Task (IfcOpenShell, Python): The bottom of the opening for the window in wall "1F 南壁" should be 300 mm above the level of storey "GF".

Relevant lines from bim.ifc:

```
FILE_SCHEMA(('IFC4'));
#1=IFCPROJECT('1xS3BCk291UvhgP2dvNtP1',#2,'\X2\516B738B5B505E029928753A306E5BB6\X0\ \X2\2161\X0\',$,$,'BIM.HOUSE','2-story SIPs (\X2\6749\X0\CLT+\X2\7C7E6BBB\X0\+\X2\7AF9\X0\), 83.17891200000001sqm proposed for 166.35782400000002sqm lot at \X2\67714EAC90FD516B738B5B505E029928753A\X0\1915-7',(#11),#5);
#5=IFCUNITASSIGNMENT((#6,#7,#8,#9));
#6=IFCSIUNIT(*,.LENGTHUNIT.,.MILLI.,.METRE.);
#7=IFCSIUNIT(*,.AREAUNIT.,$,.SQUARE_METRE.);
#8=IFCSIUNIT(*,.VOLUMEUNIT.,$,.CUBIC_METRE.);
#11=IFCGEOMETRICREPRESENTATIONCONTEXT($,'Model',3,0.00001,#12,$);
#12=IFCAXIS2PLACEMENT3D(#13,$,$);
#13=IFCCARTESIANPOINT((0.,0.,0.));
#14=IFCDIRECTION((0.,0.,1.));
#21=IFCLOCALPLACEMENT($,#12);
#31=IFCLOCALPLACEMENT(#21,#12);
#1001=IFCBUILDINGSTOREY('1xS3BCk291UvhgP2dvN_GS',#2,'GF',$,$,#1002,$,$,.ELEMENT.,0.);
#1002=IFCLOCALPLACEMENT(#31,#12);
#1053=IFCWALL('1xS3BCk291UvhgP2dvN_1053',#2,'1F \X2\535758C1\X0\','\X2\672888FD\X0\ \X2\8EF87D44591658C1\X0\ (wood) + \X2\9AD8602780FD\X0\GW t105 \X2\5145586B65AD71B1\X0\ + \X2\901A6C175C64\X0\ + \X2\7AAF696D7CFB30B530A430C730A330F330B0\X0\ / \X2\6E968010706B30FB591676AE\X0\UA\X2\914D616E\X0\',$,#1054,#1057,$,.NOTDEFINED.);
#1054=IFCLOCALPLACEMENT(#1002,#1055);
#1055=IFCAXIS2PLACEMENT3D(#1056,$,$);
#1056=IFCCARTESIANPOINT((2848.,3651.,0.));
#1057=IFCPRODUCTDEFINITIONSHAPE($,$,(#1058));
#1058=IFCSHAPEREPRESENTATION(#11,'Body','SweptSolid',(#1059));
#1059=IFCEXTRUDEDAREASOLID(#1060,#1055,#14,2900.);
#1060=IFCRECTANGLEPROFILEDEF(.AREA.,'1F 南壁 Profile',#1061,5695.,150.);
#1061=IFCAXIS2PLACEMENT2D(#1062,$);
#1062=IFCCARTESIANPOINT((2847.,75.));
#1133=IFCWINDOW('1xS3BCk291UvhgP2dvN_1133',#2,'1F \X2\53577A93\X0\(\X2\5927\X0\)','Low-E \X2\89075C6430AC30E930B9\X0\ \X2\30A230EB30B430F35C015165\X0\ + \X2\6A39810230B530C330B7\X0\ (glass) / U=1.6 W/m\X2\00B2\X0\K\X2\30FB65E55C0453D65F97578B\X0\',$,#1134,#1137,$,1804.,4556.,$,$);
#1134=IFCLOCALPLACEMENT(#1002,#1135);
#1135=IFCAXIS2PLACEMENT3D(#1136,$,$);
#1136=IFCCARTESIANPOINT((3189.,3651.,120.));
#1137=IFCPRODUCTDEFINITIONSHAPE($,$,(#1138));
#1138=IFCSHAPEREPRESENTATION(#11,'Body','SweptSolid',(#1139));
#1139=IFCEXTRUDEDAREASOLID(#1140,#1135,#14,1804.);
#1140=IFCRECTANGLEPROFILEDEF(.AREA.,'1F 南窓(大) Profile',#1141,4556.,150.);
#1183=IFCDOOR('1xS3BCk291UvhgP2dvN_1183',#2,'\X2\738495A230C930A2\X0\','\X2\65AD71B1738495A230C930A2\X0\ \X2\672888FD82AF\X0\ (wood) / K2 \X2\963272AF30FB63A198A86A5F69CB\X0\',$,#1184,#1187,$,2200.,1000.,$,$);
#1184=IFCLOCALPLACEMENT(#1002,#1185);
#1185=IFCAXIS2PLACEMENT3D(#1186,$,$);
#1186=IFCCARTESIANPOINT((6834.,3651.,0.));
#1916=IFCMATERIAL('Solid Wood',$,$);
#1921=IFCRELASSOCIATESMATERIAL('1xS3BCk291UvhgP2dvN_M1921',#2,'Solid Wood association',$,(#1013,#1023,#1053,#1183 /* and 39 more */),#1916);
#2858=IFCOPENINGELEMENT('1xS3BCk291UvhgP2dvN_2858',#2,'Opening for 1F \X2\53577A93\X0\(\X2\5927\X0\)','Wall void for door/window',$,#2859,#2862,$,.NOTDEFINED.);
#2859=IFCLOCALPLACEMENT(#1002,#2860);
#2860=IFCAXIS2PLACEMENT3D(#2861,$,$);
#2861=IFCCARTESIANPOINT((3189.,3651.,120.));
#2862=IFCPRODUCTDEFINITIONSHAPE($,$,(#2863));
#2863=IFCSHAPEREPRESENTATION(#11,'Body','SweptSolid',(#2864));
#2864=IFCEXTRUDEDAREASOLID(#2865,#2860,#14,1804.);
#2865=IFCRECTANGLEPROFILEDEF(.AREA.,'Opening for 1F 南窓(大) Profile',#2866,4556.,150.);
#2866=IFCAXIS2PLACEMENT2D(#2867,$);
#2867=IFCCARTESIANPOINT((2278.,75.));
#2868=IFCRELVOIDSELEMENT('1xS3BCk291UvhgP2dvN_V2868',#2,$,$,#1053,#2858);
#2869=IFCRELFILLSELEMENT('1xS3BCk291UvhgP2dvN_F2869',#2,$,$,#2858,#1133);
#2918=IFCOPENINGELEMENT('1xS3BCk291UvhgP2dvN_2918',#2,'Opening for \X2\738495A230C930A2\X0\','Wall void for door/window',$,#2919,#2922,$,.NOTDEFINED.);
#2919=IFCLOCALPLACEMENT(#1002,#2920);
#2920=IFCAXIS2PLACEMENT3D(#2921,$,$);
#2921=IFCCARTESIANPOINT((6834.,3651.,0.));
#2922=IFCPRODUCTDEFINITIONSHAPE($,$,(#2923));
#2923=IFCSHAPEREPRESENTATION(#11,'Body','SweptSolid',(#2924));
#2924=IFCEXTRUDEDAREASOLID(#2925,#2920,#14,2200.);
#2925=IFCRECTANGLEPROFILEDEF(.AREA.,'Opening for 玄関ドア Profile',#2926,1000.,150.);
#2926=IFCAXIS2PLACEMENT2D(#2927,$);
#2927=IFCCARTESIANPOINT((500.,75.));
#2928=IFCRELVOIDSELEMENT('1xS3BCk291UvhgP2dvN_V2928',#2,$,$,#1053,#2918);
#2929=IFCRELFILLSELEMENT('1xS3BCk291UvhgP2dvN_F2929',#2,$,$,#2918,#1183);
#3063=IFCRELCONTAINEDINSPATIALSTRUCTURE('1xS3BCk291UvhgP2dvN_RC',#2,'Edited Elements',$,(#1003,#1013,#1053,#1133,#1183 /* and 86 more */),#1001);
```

```python
import numpy as np
import ifcopenshell
import ifcopenshell.api.geometry
import ifcopenshell.geom
import ifcopenshell.util.element
import ifcopenshell.util.placement
import ifcopenshell.util.shape
import ifcopenshell.util.unit

model = ifcopenshell.open("bim.ifc")
unit_scale = ifcopenshell.util.unit.calculate_unit_scale(model)

window = model.by_guid("1xS3BCk291UvhgP2dvN_1133")
opening = window.FillsVoids[0].RelatingOpeningElement
storey = ifcopenshell.util.element.get_container(window, ifc_class="IfcBuildingStorey")
level = ifcopenshell.util.placement.get_local_placement(storey.ObjectPlacement)[2, 3]

# The opening's origin need not be at the sill, so measure its lowest point.
shape = ifcopenshell.geom.create_shape(ifcopenshell.geom.settings(), opening)
bottom = ifcopenshell.util.shape.get_shape_bottom_elevation(shape, shape.geometry) / unit_scale
dz = level + 0.3 / unit_scale - bottom

shift = np.array([0.0, 0.0, dz])
# The window is not placed relative to its opening, so move both.
for product in (opening, window):
    matrix = ifcopenshell.util.placement.get_local_placement(product.ObjectPlacement)
    matrix[:3, 3] += shift
    ifcopenshell.api.geometry.edit_object_placement(model, product=product, matrix=matrix, is_si=False)

print(f"moved by {dz * unit_scale:+.3f} m")

model.write("bim_rev.ifc")
```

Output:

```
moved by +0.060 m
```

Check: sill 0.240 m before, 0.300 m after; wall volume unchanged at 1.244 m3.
